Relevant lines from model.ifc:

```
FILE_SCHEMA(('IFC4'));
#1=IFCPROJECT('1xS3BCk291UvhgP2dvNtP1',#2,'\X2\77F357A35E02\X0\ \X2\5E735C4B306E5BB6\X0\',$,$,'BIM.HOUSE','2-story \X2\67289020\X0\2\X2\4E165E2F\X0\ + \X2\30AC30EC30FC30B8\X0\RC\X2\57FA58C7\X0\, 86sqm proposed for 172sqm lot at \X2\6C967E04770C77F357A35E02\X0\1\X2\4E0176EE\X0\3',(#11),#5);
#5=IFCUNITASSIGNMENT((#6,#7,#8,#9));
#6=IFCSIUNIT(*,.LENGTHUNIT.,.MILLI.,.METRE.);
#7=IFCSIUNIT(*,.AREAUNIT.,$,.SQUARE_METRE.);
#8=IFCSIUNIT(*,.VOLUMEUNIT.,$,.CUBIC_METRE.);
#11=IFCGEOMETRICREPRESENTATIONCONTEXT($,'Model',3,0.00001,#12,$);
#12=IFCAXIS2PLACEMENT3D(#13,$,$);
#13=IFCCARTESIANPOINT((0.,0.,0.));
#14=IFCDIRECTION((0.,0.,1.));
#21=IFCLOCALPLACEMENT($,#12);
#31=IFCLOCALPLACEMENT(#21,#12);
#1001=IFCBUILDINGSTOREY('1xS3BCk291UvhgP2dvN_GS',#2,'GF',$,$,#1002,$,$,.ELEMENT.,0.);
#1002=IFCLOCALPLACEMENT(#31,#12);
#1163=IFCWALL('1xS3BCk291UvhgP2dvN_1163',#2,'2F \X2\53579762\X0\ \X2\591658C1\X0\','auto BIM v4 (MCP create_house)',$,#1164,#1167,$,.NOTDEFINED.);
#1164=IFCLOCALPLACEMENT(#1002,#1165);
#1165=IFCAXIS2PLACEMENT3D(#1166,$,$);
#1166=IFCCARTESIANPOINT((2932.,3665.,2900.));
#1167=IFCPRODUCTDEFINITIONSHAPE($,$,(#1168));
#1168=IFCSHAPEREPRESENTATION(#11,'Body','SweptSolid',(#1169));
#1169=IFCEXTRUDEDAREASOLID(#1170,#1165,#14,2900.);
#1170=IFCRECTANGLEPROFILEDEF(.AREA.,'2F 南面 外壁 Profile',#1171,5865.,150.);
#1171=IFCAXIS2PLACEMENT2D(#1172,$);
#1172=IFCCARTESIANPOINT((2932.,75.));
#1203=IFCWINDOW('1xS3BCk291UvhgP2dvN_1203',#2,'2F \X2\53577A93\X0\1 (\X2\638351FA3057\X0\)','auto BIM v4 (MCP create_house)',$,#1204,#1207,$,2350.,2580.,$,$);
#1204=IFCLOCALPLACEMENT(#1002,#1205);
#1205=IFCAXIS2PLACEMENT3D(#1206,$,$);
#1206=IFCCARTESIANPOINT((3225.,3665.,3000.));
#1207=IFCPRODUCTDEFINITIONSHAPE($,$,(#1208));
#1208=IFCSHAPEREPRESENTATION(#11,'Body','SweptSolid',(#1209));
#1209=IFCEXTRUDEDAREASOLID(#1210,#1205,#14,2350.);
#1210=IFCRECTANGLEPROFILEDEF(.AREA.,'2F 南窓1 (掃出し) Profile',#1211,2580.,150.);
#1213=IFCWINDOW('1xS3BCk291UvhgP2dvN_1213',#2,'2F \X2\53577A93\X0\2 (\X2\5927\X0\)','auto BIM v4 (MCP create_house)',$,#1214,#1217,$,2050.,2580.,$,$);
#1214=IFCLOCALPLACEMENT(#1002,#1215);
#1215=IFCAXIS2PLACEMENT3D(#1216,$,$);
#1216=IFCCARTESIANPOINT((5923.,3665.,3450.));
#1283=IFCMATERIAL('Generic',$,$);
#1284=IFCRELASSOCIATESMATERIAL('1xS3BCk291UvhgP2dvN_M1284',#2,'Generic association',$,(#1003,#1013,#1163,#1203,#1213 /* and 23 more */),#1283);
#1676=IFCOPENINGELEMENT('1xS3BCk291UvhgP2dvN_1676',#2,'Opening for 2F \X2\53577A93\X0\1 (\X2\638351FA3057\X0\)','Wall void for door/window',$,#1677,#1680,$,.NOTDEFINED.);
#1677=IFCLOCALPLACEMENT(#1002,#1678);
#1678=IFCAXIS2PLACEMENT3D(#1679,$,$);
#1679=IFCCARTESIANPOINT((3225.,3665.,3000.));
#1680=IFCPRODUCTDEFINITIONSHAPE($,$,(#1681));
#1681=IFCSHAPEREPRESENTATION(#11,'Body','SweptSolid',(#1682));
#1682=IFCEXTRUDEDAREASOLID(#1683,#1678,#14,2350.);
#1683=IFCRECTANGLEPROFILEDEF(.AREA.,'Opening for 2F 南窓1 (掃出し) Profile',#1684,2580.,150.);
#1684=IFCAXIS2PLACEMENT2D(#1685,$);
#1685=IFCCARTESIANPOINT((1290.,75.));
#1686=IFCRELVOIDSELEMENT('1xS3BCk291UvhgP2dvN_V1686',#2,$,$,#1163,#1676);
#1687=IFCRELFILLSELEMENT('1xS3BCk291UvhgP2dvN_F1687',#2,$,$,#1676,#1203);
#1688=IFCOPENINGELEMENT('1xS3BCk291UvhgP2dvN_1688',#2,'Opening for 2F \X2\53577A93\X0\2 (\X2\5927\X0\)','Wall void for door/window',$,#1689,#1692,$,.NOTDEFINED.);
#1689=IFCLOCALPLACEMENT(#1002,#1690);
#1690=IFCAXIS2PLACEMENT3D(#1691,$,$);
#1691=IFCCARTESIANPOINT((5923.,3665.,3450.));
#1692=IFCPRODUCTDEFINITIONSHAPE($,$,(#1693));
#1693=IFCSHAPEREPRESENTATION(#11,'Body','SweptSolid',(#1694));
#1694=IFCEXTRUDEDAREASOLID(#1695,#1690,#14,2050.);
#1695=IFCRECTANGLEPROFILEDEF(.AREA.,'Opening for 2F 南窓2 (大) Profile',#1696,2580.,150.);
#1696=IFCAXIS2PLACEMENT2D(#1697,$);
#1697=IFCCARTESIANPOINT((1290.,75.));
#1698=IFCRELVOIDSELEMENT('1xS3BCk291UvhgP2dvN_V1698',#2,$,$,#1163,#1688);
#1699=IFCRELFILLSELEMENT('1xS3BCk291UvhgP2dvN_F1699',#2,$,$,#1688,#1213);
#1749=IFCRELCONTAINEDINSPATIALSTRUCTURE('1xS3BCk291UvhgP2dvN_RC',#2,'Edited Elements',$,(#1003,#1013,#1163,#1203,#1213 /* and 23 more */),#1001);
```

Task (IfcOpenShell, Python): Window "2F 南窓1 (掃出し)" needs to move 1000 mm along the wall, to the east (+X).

```python
import ifcopenshell
import ifcopenshell.api.geometry
import ifcopenshell.util.placement
import ifcopenshell.util.unit

model = ifcopenshell.open("model.ifc")
unit_scale = ifcopenshell.util.unit.calculate_unit_scale(model)

window = model.by_guid("1xS3BCk291UvhgP2dvN_1203")
opening = window.FillsVoids[0].RelatingOpeningElement
wall = opening.VoidsElements[0].RelatingBuildingElement

wall_matrix = ifcopenshell.util.placement.get_local_placement(wall.ObjectPlacement)
shift = wall_matrix[:3, 0] * 1 / unit_scale
before = ifcopenshell.util.placement.get_local_placement(window.ObjectPlacement)[:3, 3].copy()

# The window is not placed relative to its opening, so move both.
for product in (opening, window):
    matrix = ifcopenshell.util.placement.get_local_placement(product.ObjectPlacement)
    matrix[:3, 3] += shift
    ifcopenshell.api.geometry.edit_object_placement(model, product=product, matrix=matrix, is_si=False)

after = ifcopenshell.util.placement.get_local_placement(window.ObjectPlacement)[:3, 3]
print("window moved by", (after - before).round(3) + 0.0)

model.write("model_updated.ifc")
```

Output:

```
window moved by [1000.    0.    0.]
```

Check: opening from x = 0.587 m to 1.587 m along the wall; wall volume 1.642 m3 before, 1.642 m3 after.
